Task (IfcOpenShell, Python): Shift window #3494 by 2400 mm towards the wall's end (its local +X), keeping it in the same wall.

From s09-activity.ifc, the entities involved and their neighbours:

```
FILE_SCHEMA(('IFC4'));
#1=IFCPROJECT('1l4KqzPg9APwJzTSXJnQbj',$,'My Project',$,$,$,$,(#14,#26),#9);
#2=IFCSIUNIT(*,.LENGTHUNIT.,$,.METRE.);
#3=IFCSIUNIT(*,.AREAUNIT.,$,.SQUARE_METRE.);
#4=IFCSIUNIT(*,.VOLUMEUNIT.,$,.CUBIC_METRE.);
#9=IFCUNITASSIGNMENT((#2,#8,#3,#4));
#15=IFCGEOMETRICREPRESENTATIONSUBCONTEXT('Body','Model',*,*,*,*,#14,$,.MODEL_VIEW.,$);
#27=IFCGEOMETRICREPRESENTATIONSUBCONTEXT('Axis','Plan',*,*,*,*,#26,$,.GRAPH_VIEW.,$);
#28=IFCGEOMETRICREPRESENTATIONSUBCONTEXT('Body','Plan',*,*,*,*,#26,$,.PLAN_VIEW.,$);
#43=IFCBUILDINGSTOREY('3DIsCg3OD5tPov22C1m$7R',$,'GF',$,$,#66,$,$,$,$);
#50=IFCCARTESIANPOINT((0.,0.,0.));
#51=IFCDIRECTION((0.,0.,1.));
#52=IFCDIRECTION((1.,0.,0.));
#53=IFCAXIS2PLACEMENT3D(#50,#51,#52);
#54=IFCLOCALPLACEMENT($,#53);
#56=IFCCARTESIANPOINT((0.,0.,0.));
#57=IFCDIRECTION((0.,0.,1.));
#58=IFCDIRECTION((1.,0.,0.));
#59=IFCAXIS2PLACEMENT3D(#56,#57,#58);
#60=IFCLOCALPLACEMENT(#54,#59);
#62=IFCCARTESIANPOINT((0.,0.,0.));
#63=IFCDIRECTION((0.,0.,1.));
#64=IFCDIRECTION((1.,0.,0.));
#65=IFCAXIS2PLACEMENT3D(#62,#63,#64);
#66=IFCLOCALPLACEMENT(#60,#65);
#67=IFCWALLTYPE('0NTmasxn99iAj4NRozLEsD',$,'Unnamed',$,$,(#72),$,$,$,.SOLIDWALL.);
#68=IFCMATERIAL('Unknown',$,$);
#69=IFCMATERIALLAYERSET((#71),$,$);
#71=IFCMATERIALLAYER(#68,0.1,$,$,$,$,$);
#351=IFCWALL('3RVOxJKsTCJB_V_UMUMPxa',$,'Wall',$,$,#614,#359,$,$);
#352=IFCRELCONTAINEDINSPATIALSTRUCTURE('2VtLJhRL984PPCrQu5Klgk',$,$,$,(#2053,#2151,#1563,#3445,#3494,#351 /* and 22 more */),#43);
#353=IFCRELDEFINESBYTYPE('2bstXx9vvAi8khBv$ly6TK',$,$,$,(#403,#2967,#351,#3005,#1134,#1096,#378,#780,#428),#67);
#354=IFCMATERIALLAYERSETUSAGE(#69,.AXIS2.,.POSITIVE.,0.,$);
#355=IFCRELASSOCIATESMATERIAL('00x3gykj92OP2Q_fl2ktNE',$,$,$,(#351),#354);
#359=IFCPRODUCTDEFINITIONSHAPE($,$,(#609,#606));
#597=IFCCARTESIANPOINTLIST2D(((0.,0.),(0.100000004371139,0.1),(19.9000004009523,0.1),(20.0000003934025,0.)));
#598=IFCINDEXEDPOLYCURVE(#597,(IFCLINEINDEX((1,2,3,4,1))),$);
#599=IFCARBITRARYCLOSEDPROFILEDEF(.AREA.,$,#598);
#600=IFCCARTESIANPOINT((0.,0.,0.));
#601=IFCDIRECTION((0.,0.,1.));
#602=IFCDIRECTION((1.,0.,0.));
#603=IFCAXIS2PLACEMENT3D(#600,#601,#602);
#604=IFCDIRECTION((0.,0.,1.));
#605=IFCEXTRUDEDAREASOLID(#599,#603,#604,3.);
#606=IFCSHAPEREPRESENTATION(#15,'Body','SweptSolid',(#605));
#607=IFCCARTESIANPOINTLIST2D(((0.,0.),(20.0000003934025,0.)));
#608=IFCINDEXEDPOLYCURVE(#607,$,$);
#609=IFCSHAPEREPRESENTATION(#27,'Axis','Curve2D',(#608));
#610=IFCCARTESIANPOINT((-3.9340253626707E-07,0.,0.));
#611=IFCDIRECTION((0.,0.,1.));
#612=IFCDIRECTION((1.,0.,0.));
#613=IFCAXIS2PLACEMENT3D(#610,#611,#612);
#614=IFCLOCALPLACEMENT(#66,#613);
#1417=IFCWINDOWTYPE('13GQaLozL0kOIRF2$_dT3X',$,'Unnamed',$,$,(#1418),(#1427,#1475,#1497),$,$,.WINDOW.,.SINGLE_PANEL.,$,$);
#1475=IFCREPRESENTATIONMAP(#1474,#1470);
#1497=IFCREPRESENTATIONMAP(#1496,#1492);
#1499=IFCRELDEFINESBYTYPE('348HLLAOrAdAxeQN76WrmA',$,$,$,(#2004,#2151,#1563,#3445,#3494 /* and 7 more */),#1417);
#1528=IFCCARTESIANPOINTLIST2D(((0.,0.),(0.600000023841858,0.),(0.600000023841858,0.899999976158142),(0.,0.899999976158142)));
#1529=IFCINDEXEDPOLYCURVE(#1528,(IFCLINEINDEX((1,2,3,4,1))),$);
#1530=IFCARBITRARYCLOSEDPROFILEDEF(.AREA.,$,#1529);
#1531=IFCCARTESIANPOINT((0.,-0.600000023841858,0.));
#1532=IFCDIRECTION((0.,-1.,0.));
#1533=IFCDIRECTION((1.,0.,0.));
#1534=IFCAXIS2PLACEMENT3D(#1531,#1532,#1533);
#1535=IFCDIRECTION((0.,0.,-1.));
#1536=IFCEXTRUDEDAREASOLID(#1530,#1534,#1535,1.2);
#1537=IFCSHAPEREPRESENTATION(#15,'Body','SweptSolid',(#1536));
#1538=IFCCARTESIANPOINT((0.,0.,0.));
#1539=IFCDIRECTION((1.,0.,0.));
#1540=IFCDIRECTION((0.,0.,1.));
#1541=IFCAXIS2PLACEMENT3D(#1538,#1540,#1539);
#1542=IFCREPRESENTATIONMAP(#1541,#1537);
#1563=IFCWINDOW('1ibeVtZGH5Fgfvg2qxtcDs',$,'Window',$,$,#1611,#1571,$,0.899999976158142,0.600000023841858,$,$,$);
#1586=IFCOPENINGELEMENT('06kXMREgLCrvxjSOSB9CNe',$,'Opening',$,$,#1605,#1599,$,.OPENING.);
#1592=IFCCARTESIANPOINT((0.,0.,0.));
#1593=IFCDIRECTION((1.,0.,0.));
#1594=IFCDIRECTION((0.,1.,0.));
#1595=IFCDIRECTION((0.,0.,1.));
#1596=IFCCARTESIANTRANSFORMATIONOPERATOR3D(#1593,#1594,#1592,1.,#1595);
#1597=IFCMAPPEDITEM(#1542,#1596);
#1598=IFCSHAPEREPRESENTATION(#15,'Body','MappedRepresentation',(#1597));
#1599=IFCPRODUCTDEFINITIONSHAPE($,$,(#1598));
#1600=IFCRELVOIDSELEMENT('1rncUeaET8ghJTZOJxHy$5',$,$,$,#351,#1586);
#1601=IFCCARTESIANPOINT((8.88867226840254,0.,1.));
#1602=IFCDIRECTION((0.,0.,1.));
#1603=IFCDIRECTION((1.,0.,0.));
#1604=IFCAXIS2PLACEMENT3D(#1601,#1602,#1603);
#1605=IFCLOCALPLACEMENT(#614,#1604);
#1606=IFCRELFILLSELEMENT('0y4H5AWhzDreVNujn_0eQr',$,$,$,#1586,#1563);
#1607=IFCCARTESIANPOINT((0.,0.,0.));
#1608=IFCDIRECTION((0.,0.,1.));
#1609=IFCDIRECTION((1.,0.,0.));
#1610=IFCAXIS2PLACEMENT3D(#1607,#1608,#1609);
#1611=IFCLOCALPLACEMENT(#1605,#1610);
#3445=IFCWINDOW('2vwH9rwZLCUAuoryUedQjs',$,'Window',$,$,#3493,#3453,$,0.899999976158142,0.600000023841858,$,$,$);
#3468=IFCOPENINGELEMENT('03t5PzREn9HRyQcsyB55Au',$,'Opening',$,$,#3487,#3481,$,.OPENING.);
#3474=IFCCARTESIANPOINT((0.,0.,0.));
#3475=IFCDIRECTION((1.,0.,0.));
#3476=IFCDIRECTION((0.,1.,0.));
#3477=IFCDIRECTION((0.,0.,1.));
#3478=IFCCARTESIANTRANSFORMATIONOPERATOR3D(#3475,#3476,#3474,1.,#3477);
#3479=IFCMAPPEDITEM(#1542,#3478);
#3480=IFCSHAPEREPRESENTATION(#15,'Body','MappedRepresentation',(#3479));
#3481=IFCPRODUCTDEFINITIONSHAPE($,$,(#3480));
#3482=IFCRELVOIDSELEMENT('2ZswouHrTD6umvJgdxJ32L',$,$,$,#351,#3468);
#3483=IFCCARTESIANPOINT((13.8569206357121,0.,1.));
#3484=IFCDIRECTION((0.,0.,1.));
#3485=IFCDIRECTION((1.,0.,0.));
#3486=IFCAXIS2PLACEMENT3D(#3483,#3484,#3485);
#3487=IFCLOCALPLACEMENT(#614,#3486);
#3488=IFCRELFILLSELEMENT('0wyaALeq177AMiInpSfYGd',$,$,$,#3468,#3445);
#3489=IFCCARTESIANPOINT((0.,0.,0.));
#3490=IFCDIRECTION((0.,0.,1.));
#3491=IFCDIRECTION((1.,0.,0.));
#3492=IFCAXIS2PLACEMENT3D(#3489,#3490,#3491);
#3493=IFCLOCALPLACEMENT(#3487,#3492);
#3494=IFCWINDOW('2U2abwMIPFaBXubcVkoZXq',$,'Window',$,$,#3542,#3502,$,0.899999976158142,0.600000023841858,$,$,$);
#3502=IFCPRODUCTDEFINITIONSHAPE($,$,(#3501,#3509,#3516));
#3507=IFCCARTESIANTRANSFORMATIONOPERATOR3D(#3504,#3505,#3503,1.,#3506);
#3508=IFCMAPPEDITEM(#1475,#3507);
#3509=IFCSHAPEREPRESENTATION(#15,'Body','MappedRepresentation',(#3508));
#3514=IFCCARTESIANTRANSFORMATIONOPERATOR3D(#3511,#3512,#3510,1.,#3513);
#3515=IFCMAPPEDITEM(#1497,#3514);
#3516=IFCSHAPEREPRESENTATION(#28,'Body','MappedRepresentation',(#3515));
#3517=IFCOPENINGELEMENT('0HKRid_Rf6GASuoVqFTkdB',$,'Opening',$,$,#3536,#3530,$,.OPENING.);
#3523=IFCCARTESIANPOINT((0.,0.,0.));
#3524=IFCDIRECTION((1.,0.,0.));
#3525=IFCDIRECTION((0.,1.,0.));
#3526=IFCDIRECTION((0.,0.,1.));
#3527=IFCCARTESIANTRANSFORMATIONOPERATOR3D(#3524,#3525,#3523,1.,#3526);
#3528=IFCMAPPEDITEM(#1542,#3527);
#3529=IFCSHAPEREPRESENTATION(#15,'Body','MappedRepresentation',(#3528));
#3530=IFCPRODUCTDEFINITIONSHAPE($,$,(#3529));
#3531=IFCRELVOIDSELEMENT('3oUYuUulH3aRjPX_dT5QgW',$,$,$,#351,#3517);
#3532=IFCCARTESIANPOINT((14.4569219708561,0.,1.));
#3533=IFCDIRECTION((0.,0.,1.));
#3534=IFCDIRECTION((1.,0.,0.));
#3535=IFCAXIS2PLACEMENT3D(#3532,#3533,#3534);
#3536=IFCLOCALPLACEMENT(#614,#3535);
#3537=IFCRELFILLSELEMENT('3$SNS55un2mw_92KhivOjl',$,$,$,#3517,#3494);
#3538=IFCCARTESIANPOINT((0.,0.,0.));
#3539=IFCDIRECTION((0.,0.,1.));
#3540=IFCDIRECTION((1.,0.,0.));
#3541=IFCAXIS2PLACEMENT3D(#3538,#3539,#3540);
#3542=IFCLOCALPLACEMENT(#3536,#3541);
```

```python
import ifcopenshell
import ifcopenshell.api.geometry
import ifcopenshell.util.placement

model = ifcopenshell.open("s09-activity.ifc")

window = model.by_guid("2U2abwMIPFaBXubcVkoZXq")
opening = window.FillsVoids[0].RelatingOpeningElement
wall = opening.VoidsElements[0].RelatingBuildingElement

wall_matrix = ifcopenshell.util.placement.get_local_placement(wall.ObjectPlacement)
shift = wall_matrix[:3, 0] * 2.4
before = ifcopenshell.util.placement.get_local_placement(window.ObjectPlacement)[:3, 3].copy()

# The window is placed relative to its opening, so it follows when the opening moves.
matrix = ifcopenshell.util.placement.get_local_placement(opening.ObjectPlacement)
matrix[:3, 3] += shift
ifcopenshell.api.geometry.edit_object_placement(
    model, product=opening, matrix=matrix, is_si=False, should_transform_children=True
)

after = ifcopenshell.util.placement.get_local_placement(window.ObjectPlacement)[:3, 3]
print("window moved by", (after - before).round(3) + 0.0)

model.write("s09-activity_rev.ifc")
```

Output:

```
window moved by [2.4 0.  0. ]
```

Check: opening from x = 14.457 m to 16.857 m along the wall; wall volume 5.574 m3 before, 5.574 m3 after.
